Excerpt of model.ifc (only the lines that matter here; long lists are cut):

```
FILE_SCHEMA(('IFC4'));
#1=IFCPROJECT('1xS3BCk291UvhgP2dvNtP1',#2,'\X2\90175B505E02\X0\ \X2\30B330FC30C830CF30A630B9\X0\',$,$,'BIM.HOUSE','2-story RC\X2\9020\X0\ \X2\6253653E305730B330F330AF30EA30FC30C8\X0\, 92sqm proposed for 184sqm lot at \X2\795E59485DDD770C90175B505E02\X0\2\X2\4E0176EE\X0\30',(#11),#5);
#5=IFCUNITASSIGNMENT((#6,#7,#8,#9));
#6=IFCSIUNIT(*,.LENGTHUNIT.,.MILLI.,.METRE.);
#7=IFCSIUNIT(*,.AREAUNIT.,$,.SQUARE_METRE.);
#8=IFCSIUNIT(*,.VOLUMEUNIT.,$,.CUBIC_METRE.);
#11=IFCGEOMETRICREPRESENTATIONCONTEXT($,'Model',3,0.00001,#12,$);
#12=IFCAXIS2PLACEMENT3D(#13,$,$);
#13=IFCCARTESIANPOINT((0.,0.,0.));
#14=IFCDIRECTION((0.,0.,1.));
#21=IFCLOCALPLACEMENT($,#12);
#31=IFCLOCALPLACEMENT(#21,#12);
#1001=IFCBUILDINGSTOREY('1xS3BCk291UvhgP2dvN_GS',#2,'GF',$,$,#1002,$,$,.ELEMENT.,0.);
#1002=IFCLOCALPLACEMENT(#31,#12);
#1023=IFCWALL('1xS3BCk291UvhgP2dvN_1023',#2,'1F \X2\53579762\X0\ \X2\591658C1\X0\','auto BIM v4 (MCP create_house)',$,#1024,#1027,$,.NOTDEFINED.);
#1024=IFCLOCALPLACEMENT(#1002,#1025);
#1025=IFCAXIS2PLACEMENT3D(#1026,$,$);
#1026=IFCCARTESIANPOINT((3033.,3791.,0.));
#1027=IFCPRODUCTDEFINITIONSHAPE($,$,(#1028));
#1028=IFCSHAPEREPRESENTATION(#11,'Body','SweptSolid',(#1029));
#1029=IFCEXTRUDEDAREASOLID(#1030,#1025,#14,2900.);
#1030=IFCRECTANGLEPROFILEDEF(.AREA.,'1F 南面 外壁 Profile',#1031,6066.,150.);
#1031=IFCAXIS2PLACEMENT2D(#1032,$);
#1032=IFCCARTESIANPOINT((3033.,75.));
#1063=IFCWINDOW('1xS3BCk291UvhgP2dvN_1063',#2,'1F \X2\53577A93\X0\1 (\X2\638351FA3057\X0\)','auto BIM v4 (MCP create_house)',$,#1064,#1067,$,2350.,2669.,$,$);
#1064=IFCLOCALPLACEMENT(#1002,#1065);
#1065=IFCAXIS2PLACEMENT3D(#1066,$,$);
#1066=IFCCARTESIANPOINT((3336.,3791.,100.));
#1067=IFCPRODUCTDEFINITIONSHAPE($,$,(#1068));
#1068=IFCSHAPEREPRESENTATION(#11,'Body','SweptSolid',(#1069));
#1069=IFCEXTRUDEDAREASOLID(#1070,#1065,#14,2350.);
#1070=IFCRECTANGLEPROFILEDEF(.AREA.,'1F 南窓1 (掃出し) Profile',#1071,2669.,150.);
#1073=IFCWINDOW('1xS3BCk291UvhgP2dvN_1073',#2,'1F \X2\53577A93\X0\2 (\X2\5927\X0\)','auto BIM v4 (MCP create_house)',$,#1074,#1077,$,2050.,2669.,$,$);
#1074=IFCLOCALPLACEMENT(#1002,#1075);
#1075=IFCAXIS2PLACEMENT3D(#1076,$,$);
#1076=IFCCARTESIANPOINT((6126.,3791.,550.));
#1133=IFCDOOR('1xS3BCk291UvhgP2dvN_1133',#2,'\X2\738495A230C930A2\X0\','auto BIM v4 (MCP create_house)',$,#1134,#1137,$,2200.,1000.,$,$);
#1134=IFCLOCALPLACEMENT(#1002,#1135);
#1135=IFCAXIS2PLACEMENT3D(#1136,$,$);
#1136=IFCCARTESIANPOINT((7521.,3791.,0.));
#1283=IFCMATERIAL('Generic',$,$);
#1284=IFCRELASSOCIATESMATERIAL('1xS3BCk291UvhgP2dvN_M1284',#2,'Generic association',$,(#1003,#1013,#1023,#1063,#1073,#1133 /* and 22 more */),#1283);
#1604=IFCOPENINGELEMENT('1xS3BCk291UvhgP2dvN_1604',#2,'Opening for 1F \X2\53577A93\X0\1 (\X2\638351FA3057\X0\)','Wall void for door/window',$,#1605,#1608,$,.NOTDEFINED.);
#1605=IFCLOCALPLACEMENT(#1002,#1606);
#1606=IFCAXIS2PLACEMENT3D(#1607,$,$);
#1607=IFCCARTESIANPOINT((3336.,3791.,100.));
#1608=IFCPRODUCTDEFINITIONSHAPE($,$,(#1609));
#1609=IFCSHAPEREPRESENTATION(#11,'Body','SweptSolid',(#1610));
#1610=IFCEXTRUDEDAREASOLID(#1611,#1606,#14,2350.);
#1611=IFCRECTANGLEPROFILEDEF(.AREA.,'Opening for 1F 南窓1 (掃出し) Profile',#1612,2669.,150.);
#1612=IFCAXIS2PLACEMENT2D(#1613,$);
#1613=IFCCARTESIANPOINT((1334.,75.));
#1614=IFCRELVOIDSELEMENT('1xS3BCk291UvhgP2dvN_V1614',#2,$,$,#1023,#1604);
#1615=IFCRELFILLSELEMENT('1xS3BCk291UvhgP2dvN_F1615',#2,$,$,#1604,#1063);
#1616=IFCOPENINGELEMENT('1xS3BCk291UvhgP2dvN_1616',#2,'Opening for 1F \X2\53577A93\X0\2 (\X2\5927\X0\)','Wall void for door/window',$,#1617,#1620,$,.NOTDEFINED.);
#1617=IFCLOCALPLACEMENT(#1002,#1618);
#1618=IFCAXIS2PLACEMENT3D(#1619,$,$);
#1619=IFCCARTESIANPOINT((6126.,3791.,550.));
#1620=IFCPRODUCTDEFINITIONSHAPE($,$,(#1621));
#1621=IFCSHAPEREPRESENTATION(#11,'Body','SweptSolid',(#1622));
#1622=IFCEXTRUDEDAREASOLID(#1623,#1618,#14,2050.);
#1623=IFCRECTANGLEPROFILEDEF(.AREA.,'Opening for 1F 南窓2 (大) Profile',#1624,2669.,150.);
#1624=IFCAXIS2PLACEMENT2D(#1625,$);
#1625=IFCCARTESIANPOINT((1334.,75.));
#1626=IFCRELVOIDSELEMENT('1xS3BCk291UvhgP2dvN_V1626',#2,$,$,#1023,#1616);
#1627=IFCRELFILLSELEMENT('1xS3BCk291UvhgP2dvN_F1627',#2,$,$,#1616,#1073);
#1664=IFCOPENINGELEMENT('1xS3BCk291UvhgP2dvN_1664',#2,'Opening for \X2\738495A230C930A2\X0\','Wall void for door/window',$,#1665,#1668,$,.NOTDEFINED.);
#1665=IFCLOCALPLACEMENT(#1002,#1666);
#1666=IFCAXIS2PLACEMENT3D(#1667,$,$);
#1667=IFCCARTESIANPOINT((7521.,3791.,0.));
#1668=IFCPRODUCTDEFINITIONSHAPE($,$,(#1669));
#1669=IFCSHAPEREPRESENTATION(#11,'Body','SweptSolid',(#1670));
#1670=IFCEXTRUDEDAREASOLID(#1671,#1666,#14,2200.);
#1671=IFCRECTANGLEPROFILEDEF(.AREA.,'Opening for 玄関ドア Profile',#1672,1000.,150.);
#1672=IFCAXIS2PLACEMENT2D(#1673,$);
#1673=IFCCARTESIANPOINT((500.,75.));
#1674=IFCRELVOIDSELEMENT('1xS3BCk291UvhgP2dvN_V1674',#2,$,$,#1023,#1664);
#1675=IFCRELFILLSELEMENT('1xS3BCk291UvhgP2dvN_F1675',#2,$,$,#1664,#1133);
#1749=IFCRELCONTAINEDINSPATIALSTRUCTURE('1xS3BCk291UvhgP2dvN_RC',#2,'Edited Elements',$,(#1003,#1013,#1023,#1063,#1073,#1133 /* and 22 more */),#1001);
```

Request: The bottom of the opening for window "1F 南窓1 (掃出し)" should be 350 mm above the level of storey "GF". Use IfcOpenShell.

```python
import numpy as np
import ifcopenshell
import ifcopenshell.api.geometry
import ifcopenshell.geom
import ifcopenshell.util.element
import ifcopenshell.util.placement
import ifcopenshell.util.shape
import ifcopenshell.util.unit

model = ifcopenshell.open("model.ifc")
unit_scale = ifcopenshell.util.unit.calculate_unit_scale(model)

window = model.by_id(1063)
opening = window.FillsVoids[0].RelatingOpeningElement
storey = ifcopenshell.util.element.get_container(window, ifc_class="IfcBuildingStorey")
level = ifcopenshell.util.placement.get_local_placement(storey.ObjectPlacement)[2, 3]

# The opening's origin need not be at the sill, so measure its lowest point.
shape = ifcopenshell.geom.create_shape(ifcopenshell.geom.settings(), opening)
bottom = ifcopenshell.util.shape.get_shape_bottom_elevation(shape, shape.geometry) / unit_scale
dz = level + 0.35 / unit_scale - bottom

shift = np.array([0.0, 0.0, dz])
# The window is not placed relative to its opening, so move both.
for product in (opening, window):
    matrix = ifcopenshell.util.placement.get_local_placement(product.ObjectPlacement)
    matrix[:3, 3] += shift
    ifcopenshell.api.geometry.edit_object_placement(model, product=product, matrix=matrix, is_si=False)

print(f"moved by {dz * unit_scale:+.3f} m")

model.write("model_edited.ifc")
```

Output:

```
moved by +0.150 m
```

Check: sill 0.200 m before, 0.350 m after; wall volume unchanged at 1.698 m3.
